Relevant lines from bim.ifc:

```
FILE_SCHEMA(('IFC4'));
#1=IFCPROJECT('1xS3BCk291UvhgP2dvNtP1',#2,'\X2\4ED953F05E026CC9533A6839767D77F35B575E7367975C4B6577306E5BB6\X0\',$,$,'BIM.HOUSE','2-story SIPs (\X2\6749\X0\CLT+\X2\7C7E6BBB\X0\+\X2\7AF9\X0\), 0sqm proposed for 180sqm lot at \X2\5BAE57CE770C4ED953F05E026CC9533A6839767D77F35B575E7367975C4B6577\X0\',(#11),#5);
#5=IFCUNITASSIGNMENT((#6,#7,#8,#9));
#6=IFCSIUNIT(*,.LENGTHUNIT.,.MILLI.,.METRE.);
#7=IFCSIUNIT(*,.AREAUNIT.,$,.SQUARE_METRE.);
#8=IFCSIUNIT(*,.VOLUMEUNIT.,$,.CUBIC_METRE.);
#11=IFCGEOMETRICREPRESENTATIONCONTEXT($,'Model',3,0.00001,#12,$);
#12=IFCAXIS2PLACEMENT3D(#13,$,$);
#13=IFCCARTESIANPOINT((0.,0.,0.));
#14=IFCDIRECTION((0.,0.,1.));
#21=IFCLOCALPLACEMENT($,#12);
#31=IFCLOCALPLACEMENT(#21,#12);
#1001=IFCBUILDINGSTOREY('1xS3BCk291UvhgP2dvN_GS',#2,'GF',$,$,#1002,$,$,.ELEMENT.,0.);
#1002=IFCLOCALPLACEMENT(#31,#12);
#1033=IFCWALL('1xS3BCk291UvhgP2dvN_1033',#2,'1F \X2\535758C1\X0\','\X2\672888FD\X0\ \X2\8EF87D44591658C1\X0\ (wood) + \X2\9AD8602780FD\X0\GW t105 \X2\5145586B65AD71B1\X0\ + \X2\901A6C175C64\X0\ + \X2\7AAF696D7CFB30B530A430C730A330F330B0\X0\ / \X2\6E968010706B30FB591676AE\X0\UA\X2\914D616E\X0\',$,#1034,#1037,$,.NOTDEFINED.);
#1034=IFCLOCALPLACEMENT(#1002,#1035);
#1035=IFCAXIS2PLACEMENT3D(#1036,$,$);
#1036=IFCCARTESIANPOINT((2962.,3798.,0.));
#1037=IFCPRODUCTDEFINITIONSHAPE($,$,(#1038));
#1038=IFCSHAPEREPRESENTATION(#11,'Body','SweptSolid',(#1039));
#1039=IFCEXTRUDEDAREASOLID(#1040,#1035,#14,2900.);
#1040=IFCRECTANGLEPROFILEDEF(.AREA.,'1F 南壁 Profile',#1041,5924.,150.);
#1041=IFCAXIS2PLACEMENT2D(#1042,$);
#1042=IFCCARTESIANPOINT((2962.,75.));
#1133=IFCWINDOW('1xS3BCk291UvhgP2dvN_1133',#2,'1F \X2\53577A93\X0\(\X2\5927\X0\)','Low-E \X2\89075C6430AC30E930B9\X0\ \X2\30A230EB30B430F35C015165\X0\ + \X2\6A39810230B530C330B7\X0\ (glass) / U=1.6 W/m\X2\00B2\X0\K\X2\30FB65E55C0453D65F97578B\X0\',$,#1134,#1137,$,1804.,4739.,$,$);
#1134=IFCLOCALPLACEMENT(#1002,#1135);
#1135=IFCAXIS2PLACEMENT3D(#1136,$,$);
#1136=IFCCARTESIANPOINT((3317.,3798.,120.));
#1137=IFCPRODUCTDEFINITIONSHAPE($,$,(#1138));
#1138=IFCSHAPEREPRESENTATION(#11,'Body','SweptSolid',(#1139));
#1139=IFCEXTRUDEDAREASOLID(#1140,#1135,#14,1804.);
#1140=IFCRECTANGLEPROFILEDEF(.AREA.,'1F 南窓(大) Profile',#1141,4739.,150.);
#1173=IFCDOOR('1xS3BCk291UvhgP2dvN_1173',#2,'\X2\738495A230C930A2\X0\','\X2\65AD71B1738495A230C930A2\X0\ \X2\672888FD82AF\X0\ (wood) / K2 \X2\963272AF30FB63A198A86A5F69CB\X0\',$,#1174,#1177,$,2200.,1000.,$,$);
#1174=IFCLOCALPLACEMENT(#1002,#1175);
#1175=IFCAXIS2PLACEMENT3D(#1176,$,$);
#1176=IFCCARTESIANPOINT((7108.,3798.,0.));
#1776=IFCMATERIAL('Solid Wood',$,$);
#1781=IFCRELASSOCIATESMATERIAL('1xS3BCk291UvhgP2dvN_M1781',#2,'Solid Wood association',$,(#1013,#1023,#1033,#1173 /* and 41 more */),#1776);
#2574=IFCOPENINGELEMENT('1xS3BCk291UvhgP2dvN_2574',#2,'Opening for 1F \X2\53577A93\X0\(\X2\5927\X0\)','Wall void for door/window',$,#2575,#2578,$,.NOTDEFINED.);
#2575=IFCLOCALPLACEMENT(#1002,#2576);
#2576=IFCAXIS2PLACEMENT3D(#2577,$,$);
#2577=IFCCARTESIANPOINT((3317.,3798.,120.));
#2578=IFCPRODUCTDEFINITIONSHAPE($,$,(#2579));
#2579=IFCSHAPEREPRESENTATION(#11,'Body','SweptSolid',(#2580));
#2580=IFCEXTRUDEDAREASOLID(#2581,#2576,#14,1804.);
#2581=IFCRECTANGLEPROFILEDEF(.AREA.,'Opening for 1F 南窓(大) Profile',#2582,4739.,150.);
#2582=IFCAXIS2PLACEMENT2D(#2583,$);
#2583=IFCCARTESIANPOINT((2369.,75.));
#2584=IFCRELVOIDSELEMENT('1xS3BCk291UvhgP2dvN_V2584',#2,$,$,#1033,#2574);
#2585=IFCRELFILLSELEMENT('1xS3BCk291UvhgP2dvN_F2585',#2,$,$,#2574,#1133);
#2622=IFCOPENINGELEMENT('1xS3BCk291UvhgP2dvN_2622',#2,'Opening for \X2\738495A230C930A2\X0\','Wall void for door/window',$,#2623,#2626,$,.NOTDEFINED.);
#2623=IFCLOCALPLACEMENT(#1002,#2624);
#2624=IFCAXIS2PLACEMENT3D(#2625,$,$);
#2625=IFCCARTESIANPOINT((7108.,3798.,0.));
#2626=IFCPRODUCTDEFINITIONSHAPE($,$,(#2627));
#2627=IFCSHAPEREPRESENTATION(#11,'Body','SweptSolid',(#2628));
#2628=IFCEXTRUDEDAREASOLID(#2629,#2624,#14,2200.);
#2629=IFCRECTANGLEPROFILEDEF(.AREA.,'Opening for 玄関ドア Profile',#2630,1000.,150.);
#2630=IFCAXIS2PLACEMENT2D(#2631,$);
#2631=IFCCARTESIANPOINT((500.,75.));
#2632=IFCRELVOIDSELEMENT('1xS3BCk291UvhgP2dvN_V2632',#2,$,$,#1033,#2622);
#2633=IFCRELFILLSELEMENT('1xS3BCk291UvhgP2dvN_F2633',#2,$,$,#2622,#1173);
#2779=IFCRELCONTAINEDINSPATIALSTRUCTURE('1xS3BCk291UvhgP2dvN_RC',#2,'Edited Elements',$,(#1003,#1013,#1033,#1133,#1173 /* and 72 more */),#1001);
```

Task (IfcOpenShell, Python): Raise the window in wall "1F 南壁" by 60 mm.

```python
import numpy as np
import ifcopenshell
import ifcopenshell.api.geometry
import ifcopenshell.util.placement
import ifcopenshell.util.unit

model = ifcopenshell.open("bim.ifc")
unit_scale = ifcopenshell.util.unit.calculate_unit_scale(model)

window = model.by_guid("1xS3BCk291UvhgP2dvN_1133")
opening = window.FillsVoids[0].RelatingOpeningElement
dz = 60.0

shift = np.array([0.0, 0.0, dz])
# The window is not placed relative to its opening, so move both.
for product in (opening, window):
    matrix = ifcopenshell.util.placement.get_local_placement(product.ObjectPlacement)
    matrix[:3, 3] += shift
    ifcopenshell.api.geometry.edit_object_placement(model, product=product, matrix=matrix, is_si=False)

print(f"moved by {dz * unit_scale:+.3f} m")

model.write("bim_edited.ifc")
```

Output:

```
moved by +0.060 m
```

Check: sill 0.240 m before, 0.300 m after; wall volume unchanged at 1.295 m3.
